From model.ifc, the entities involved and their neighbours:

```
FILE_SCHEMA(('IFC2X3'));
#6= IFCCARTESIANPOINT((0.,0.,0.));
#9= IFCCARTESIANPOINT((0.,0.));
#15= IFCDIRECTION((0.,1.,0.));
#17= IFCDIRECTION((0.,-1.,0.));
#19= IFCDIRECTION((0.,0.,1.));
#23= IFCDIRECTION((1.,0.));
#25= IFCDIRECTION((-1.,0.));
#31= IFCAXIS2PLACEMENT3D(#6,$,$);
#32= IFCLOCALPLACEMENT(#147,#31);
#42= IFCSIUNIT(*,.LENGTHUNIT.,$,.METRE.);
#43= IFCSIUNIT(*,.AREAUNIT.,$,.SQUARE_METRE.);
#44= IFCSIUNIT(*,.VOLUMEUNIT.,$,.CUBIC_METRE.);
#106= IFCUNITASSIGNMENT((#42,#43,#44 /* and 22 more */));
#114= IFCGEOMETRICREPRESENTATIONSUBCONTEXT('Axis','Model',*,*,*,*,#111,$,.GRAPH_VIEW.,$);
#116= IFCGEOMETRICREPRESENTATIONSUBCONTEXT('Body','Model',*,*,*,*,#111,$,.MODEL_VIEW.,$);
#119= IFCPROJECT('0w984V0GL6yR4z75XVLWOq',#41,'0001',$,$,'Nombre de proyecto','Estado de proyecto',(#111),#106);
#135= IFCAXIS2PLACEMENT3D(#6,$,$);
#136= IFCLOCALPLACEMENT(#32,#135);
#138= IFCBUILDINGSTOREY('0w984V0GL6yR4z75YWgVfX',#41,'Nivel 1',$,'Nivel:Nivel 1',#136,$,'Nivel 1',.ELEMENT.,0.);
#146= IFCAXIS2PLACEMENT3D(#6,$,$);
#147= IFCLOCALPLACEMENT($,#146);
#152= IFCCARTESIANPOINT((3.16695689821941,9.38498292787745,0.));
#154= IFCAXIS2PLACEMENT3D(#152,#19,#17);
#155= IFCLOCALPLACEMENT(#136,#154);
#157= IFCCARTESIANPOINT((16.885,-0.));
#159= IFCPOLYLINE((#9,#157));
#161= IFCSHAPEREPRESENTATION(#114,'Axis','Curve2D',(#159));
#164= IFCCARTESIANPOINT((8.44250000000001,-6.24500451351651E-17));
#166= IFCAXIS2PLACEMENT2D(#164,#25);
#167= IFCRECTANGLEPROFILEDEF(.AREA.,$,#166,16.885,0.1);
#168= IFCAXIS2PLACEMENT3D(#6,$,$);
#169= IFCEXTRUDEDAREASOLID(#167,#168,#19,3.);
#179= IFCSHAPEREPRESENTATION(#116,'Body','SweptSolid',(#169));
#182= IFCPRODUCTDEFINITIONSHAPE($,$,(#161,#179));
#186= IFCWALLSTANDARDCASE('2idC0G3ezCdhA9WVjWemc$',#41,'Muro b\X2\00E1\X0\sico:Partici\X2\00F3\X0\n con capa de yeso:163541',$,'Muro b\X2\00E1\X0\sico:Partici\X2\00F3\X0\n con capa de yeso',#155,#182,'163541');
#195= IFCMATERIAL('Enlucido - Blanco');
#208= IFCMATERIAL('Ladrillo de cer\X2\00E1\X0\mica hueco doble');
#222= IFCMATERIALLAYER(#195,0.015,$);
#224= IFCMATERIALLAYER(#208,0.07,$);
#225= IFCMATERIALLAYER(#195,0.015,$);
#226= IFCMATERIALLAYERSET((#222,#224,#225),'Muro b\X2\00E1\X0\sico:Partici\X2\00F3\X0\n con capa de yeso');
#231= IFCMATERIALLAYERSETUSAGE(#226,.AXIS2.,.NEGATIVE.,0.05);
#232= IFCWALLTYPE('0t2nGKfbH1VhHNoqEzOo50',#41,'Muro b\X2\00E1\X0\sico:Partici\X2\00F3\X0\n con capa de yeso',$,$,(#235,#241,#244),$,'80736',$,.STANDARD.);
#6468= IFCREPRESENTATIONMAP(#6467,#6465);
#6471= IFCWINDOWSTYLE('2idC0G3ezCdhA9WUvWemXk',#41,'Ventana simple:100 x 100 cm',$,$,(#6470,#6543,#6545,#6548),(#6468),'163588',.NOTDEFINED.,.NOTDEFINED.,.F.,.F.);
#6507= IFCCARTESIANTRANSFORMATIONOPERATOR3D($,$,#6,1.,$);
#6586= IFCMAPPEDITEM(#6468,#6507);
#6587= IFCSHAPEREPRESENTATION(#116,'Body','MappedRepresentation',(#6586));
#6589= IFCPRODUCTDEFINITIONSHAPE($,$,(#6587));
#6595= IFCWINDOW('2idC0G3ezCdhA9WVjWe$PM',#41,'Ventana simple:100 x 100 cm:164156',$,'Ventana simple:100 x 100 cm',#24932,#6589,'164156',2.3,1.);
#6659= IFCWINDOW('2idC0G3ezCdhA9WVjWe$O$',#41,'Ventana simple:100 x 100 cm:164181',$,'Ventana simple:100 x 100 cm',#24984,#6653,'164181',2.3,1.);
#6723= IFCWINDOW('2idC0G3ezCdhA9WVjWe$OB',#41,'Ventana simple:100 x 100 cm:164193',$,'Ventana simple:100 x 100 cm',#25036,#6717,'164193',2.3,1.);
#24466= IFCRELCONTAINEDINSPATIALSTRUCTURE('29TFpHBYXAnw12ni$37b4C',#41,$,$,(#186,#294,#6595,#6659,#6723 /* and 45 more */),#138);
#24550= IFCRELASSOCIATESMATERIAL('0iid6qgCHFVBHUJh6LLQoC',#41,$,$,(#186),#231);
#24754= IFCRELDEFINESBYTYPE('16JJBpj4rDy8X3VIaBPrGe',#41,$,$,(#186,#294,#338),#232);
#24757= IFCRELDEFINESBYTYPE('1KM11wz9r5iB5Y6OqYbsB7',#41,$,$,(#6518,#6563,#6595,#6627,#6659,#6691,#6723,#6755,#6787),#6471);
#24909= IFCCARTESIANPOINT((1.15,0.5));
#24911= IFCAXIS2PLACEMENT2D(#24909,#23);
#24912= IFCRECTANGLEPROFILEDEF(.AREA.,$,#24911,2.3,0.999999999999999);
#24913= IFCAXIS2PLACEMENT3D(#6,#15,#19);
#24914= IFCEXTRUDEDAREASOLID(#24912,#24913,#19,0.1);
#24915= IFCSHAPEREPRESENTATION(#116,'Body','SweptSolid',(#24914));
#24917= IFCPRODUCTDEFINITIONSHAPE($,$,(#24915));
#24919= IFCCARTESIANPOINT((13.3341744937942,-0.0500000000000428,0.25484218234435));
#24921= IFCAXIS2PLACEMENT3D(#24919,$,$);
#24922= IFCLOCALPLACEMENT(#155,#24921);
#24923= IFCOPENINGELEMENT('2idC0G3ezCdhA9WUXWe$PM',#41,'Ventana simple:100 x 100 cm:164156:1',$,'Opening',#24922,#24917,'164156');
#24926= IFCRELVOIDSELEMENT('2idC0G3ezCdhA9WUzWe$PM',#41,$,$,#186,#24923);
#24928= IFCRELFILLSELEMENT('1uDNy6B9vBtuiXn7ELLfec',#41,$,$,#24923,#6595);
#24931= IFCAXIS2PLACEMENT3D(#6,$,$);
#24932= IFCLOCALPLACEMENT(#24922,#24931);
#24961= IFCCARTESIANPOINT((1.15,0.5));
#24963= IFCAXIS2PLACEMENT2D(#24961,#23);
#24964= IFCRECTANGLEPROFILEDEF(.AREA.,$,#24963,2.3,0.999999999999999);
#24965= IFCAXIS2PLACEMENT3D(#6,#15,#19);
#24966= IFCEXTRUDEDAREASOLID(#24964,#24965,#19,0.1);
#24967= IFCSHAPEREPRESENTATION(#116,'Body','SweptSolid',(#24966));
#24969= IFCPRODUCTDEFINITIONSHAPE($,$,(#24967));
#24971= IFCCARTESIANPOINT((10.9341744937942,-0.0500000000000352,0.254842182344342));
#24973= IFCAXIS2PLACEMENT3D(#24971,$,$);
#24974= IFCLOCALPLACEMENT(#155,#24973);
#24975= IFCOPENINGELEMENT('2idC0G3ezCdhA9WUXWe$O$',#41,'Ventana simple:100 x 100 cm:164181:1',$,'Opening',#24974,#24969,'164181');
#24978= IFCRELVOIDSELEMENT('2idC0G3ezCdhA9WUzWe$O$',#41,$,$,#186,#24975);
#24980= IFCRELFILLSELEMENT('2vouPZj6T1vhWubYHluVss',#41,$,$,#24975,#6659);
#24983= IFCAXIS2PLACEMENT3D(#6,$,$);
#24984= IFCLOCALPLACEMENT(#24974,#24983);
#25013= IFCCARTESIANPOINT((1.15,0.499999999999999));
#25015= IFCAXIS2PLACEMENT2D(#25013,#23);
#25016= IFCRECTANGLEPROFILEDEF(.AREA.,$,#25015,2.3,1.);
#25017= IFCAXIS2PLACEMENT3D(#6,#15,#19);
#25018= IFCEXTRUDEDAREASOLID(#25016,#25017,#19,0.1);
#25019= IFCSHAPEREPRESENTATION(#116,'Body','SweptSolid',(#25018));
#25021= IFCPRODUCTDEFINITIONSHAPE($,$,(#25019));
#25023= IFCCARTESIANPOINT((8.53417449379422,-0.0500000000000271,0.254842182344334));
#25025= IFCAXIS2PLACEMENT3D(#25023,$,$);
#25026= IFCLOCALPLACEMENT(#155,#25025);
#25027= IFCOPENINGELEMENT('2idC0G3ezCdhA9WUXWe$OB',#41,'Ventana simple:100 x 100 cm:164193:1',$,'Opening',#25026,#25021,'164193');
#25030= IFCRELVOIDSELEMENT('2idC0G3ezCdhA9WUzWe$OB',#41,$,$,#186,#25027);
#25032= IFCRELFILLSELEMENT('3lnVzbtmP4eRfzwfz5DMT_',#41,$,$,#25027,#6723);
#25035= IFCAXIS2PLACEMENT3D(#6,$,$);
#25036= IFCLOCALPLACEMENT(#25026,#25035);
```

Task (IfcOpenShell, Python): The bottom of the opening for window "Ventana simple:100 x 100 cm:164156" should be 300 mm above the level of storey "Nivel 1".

```python
import numpy as np
import ifcopenshell
import ifcopenshell.api.geometry
import ifcopenshell.geom
import ifcopenshell.util.element
import ifcopenshell.util.placement
import ifcopenshell.util.shape
import ifcopenshell.util.unit

model = ifcopenshell.open("model.ifc")
unit_scale = ifcopenshell.util.unit.calculate_unit_scale(model)

window = model.by_guid("2idC0G3ezCdhA9WVjWe$PM")
opening = window.FillsVoids[0].RelatingOpeningElement
storey = ifcopenshell.util.element.get_container(window, ifc_class="IfcBuildingStorey")
level = ifcopenshell.util.placement.get_local_placement(storey.ObjectPlacement)[2, 3]

# The opening's origin need not be at the sill, so measure its lowest point.
shape = ifcopenshell.geom.create_shape(ifcopenshell.geom.settings(), opening)
bottom = ifcopenshell.util.shape.get_shape_bottom_elevation(shape, shape.geometry) / unit_scale
dz = level + 0.3 - bottom

shift = np.array([0.0, 0.0, dz])
# The window is placed relative to its opening, so it follows when the opening moves.
matrix = ifcopenshell.util.placement.get_local_placement(opening.ObjectPlacement)
matrix[:3, 3] += shift
ifcopenshell.api.geometry.edit_object_placement(
    model, product=opening, matrix=matrix, is_si=False, should_transform_children=True
)

print(f"moved by {dz * unit_scale:+.3f} m")

model.write("model_rev.ifc")
```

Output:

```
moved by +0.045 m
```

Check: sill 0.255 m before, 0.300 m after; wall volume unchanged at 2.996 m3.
